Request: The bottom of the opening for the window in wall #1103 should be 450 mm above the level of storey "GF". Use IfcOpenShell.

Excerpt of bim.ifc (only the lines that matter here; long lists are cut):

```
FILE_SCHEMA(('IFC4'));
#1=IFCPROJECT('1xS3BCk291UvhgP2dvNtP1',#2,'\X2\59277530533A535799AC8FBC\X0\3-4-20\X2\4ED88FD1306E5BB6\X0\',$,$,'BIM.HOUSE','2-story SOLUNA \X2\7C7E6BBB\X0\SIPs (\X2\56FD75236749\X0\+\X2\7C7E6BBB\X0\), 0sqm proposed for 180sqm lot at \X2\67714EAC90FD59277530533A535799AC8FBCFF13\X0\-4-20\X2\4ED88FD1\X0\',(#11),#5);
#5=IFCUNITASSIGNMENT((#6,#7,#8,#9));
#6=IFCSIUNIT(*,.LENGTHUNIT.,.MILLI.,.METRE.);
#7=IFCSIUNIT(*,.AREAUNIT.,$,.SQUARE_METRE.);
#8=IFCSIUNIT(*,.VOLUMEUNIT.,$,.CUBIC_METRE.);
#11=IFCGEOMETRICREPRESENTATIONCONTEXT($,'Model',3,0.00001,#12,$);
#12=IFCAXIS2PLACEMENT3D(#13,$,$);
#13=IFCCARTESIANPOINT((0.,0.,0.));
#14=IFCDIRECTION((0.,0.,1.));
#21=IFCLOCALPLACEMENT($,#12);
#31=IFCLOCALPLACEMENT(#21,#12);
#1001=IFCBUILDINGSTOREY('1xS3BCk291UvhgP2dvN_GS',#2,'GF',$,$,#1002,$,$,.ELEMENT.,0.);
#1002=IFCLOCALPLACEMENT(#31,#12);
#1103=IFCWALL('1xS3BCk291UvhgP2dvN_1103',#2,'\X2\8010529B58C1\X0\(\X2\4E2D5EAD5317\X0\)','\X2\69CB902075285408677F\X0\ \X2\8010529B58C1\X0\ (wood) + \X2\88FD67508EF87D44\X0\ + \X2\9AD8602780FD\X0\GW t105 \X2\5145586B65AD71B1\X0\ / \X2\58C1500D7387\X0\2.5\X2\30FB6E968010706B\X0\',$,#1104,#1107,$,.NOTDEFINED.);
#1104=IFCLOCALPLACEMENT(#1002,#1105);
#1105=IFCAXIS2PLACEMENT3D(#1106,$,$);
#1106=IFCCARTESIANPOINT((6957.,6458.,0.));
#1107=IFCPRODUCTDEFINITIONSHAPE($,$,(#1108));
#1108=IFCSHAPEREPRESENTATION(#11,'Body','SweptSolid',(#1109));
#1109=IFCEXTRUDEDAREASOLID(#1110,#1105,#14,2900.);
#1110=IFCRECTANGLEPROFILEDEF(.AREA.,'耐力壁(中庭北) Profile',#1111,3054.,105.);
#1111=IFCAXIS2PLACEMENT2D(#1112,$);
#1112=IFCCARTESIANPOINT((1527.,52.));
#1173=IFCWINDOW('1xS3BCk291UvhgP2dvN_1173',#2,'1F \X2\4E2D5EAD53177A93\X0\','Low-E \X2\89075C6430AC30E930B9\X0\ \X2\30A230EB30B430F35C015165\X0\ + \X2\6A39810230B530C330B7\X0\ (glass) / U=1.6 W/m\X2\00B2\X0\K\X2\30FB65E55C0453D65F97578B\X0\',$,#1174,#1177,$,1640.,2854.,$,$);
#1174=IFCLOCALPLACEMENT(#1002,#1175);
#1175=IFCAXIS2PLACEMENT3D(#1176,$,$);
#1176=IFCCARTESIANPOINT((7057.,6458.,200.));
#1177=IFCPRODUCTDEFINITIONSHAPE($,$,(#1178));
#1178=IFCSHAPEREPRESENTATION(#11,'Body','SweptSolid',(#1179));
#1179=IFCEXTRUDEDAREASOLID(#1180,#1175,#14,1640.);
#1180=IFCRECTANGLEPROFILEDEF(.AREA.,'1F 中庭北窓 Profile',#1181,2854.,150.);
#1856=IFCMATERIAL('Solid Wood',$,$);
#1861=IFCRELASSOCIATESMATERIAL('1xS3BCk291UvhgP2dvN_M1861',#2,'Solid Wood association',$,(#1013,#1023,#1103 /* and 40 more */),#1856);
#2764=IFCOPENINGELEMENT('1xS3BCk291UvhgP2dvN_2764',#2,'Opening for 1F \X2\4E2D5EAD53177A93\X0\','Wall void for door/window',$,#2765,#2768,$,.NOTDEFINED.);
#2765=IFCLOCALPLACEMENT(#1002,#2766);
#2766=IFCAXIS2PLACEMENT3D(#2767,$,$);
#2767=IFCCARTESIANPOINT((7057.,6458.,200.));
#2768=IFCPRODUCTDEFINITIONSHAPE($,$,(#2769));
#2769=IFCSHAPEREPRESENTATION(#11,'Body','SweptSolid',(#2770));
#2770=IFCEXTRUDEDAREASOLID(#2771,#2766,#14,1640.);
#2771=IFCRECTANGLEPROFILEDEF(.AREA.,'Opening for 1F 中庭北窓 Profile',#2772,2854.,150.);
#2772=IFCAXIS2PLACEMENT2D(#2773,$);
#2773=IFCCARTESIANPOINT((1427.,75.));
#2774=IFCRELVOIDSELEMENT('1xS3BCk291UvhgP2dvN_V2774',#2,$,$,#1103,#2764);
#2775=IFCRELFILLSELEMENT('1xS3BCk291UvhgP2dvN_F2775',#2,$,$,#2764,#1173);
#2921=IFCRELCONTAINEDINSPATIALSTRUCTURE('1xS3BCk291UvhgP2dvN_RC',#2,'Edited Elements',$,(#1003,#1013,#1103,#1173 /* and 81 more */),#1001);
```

```python
import numpy as np
import ifcopenshell
import ifcopenshell.api.geometry
import ifcopenshell.geom
import ifcopenshell.util.element
import ifcopenshell.util.placement
import ifcopenshell.util.shape
import ifcopenshell.util.unit

model = ifcopenshell.open("bim.ifc")
unit_scale = ifcopenshell.util.unit.calculate_unit_scale(model)

window = model.by_guid("1xS3BCk291UvhgP2dvN_1173")
opening = window.FillsVoids[0].RelatingOpeningElement
storey = ifcopenshell.util.element.get_container(window, ifc_class="IfcBuildingStorey")
level = ifcopenshell.util.placement.get_local_placement(storey.ObjectPlacement)[2, 3]

# The opening's origin need not be at the sill, so measure its lowest point.
shape = ifcopenshell.geom.create_shape(ifcopenshell.geom.settings(), opening)
bottom = ifcopenshell.util.shape.get_shape_bottom_elevation(shape, shape.geometry) / unit_scale
dz = level + 0.45 / unit_scale - bottom

shift = np.array([0.0, 0.0, dz])
# The window is not placed relative to its opening, so move both.
for product in (opening, window):
    matrix = ifcopenshell.util.placement.get_local_placement(product.ObjectPlacement)
    matrix[:3, 3] += shift
    ifcopenshell.api.geometry.edit_object_placement(model, product=product, matrix=matrix, is_si=False)

print(f"moved by {dz * unit_scale:+.3f} m")

model.write("bim_updated.ifc")
```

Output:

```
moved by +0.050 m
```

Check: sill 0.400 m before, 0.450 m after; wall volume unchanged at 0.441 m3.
